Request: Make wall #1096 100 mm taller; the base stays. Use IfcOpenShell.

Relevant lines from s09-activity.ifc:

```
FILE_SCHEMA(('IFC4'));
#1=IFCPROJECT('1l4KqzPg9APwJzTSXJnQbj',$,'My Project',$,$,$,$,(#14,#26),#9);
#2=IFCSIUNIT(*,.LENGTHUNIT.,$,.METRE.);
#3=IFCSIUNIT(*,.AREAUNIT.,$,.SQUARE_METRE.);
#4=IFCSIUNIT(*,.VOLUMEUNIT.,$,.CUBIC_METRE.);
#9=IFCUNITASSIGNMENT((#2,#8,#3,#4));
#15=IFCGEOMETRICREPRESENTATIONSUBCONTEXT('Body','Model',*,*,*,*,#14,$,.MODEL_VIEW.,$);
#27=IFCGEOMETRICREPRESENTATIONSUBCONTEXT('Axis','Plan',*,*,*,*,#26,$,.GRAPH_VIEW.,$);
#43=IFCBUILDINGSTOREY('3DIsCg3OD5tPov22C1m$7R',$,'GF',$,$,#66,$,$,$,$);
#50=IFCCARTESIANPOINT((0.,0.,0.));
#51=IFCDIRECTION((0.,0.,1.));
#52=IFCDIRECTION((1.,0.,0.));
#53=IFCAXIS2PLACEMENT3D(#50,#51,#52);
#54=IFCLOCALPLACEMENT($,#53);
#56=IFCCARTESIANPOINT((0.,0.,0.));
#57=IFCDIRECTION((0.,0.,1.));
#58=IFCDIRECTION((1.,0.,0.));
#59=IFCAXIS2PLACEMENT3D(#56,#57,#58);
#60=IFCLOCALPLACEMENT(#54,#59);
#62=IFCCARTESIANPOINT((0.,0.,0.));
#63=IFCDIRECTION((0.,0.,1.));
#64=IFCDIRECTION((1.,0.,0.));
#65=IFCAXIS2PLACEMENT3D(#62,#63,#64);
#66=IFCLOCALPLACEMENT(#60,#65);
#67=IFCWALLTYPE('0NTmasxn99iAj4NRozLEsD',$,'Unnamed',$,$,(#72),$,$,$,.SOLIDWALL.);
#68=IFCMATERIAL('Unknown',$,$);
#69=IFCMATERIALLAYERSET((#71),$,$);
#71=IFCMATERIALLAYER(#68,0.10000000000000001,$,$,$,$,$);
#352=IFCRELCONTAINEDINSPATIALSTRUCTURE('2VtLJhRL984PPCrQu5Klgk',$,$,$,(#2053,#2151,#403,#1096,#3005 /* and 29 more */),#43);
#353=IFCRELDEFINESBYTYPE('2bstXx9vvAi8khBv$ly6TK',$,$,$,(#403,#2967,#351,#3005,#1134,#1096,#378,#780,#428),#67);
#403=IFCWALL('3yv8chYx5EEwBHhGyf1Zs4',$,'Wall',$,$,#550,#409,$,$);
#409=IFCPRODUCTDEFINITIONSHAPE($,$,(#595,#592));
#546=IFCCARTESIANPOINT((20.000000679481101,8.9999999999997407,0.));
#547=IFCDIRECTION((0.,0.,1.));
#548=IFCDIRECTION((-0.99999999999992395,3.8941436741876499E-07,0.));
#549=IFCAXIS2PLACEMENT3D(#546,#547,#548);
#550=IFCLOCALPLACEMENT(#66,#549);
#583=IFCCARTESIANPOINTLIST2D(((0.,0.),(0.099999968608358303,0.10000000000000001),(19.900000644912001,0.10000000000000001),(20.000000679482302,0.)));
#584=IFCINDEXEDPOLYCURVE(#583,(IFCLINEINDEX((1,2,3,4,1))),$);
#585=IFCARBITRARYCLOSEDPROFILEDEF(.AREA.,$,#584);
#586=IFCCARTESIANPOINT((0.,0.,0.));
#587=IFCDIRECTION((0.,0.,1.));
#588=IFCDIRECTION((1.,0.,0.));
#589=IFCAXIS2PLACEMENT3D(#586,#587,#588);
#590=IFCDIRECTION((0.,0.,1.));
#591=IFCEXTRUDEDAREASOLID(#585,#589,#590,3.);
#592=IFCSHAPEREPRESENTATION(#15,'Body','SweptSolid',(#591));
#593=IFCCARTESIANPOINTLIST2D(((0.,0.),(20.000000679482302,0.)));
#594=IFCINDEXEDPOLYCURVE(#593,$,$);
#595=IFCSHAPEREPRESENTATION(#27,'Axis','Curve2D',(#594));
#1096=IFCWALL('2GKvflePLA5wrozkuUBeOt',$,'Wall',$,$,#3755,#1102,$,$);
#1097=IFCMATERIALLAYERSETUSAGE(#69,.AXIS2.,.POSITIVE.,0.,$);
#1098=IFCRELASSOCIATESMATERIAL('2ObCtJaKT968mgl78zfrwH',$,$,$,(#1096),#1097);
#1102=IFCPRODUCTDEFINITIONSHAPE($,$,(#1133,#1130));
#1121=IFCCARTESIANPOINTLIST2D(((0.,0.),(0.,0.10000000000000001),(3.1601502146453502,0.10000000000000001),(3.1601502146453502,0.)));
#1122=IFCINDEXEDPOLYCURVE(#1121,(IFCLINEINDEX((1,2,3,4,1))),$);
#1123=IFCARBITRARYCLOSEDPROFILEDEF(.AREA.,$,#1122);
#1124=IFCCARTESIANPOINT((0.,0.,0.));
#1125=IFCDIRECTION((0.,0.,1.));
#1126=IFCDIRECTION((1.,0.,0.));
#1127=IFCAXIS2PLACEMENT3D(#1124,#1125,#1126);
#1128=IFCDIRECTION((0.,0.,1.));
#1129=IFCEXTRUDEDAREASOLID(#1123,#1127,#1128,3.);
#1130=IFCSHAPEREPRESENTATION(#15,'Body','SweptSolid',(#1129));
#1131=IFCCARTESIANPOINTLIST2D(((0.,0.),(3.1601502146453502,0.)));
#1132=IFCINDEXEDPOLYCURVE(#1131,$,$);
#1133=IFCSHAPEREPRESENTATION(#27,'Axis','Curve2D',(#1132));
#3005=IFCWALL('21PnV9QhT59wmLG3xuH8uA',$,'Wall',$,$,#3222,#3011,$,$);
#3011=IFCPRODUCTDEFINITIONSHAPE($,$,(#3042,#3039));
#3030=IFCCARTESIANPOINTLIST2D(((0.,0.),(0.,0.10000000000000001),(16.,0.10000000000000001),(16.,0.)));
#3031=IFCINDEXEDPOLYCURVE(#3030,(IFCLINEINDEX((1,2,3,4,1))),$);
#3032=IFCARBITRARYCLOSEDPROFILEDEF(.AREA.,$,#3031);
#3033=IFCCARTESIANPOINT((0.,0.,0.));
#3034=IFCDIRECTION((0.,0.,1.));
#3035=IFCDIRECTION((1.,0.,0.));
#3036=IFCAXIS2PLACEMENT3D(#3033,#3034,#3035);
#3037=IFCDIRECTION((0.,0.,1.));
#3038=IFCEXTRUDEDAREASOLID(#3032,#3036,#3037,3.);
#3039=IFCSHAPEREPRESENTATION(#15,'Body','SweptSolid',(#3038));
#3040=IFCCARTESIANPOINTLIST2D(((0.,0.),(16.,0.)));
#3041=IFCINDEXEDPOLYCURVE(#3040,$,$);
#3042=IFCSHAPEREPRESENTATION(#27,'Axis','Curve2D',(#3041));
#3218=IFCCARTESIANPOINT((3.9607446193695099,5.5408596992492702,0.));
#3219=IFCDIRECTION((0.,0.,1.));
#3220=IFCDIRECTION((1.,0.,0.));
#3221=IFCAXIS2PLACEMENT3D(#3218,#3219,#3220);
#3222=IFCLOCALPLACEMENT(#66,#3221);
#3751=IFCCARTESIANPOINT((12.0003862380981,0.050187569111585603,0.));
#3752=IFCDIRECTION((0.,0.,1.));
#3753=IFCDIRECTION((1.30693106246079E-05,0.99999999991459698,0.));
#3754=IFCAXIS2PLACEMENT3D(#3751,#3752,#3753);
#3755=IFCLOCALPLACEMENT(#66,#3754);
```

```python
import ifcopenshell
import ifcopenshell.geom
import ifcopenshell.util.representation
import ifcopenshell.util.shape

model = ifcopenshell.open("s09-activity.ifc")
settings = ifcopenshell.geom.settings()


def volume(element):
    """Net volume in cubic metres, openings subtracted."""
    shape = ifcopenshell.geom.create_shape(settings, element)
    return ifcopenshell.util.shape.get_volume(shape.geometry)


wall = model.by_guid("2GKvflePLA5wrozkuUBeOt")
before = volume(wall)

body = ifcopenshell.util.representation.get_representation(wall, "Model", "Body")
solid = body.Items[0]
old_height = solid.Depth
solid.Depth += 0.1
after = volume(wall)

print(f"height {old_height:g} -> {solid.Depth:g}, volume {before:.3f} -> {after:.3f} m3")

model.write("s09-activity-out.ifc")
```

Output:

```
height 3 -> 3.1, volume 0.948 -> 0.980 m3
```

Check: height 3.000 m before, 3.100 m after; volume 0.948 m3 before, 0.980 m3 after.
